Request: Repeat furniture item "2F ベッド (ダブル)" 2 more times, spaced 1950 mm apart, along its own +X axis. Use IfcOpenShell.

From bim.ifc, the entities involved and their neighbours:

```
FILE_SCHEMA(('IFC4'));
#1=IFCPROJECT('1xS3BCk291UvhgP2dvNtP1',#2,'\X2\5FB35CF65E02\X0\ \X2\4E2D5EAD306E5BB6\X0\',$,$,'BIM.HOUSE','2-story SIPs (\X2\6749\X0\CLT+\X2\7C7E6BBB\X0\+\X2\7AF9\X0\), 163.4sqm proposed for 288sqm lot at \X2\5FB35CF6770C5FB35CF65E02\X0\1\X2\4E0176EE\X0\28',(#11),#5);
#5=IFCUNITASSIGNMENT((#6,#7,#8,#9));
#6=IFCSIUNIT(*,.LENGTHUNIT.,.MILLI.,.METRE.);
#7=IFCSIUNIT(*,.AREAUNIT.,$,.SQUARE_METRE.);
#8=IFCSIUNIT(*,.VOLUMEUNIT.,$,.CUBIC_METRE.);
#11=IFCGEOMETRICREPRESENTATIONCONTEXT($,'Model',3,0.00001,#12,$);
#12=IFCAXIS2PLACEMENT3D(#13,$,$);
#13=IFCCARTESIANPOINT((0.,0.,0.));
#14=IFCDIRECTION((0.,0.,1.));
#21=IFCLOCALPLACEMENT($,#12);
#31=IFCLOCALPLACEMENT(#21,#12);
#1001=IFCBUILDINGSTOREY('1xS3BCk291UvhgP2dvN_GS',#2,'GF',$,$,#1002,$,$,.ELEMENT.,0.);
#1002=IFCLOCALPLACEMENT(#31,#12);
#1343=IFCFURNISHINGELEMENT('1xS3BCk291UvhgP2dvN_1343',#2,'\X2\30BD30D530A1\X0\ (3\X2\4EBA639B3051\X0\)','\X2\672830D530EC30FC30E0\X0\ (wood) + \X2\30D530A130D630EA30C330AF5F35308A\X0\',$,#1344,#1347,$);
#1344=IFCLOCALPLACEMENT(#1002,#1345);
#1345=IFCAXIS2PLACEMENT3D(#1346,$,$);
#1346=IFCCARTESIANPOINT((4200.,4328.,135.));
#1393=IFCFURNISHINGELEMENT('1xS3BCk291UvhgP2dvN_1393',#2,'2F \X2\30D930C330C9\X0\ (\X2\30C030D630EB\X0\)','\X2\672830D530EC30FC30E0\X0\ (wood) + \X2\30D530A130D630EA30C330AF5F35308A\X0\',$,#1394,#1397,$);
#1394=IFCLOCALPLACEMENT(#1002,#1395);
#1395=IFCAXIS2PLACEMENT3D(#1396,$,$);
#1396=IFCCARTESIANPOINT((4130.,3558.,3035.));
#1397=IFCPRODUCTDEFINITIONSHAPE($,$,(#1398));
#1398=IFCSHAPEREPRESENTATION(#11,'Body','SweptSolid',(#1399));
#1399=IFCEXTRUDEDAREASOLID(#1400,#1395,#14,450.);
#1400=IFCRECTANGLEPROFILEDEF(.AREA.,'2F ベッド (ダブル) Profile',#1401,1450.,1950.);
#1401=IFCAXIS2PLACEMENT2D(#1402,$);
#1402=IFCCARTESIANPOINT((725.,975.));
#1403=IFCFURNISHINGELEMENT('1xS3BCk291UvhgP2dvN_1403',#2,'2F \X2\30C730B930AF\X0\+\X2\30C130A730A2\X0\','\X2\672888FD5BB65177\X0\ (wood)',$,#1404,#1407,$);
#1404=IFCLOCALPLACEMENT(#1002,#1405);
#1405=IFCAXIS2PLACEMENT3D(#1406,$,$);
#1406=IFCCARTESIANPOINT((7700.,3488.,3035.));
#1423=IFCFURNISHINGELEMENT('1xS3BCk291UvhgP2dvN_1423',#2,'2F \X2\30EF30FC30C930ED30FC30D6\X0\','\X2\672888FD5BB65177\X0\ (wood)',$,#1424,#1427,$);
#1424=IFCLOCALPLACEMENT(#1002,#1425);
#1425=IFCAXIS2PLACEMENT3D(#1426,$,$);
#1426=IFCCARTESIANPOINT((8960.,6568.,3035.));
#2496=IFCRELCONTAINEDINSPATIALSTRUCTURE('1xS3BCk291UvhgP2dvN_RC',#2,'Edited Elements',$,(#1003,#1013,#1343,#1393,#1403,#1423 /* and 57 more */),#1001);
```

```python
import ifcopenshell
import ifcopenshell.api.geometry
import ifcopenshell.api.root
import ifcopenshell.util.element
import ifcopenshell.util.placement

model = ifcopenshell.open("bim.ifc")


def reuse_history(source, copy):
    """copy_class also copies each property set's owner history, people and application; keep the originals."""
    for rel in copy.IsDefinedBy:
        if rel.is_a("IfcRelDefinesByProperties") and (history := rel.RelatingPropertyDefinition.OwnerHistory):
            rel.RelatingPropertyDefinition.OwnerHistory = source.OwnerHistory
            ifcopenshell.util.element.remove_deep2(model, history)


source = model.by_guid("1xS3BCk291UvhgP2dvN_1393")
base = ifcopenshell.util.placement.get_local_placement(source.ObjectPlacement)
step = base[:3, 0] * 1950.0

for i in range(1, 3):
    copy = ifcopenshell.api.root.copy_class(model, product=source)
    copy.Representation = ifcopenshell.util.element.copy_deep(
        model, source.Representation, exclude=["IfcGeometricRepresentationContext", "IfcRepresentationMap"]
    )
    reuse_history(source, copy)
    matrix = base.copy()
    matrix[:3, 3] += i * step
    print("added at", matrix[:3, 3].round(3) + 0.0)
    ifcopenshell.api.geometry.edit_object_placement(model, product=copy, matrix=matrix, is_si=False)

model.write("bim_rev.ifc")
```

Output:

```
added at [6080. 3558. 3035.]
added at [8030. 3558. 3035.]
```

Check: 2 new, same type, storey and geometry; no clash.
